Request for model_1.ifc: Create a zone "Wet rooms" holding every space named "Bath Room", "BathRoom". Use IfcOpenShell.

First a look at what the model holds.

```python
import ifcopenshell

model = ifcopenshell.open("model_1.ifc")
print(model.schema)
seen = {}
for space in model.by_type("IfcSpace"):
    seen[space.LongName] = seen.get(space.LongName, 0) + 1
for name, count in sorted(seen.items(), key=str):
    print(count, "x", name)
print("zones:", [z.Name for z in model.by_type("IfcZone")][:20])
```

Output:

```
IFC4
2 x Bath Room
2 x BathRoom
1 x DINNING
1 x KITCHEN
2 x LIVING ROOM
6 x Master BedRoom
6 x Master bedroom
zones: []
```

```python
import ifcopenshell
import ifcopenshell.api.group
import ifcopenshell.api.root

model = ifcopenshell.open("model_1.ifc")

names = {"Bath Room", "BathRoom"}
spaces = [s for s in model.by_type("IfcSpace") if s.LongName in names]

zone = ifcopenshell.api.root.create_entity(model, ifc_class="IfcZone", name="Wet rooms")
ifcopenshell.api.group.assign_group(model, products=spaces, group=zone)
print(len(spaces), "spaces in", zone.Name)

model.write("model_1_edited.ifc")
```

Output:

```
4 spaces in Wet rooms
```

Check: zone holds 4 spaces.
